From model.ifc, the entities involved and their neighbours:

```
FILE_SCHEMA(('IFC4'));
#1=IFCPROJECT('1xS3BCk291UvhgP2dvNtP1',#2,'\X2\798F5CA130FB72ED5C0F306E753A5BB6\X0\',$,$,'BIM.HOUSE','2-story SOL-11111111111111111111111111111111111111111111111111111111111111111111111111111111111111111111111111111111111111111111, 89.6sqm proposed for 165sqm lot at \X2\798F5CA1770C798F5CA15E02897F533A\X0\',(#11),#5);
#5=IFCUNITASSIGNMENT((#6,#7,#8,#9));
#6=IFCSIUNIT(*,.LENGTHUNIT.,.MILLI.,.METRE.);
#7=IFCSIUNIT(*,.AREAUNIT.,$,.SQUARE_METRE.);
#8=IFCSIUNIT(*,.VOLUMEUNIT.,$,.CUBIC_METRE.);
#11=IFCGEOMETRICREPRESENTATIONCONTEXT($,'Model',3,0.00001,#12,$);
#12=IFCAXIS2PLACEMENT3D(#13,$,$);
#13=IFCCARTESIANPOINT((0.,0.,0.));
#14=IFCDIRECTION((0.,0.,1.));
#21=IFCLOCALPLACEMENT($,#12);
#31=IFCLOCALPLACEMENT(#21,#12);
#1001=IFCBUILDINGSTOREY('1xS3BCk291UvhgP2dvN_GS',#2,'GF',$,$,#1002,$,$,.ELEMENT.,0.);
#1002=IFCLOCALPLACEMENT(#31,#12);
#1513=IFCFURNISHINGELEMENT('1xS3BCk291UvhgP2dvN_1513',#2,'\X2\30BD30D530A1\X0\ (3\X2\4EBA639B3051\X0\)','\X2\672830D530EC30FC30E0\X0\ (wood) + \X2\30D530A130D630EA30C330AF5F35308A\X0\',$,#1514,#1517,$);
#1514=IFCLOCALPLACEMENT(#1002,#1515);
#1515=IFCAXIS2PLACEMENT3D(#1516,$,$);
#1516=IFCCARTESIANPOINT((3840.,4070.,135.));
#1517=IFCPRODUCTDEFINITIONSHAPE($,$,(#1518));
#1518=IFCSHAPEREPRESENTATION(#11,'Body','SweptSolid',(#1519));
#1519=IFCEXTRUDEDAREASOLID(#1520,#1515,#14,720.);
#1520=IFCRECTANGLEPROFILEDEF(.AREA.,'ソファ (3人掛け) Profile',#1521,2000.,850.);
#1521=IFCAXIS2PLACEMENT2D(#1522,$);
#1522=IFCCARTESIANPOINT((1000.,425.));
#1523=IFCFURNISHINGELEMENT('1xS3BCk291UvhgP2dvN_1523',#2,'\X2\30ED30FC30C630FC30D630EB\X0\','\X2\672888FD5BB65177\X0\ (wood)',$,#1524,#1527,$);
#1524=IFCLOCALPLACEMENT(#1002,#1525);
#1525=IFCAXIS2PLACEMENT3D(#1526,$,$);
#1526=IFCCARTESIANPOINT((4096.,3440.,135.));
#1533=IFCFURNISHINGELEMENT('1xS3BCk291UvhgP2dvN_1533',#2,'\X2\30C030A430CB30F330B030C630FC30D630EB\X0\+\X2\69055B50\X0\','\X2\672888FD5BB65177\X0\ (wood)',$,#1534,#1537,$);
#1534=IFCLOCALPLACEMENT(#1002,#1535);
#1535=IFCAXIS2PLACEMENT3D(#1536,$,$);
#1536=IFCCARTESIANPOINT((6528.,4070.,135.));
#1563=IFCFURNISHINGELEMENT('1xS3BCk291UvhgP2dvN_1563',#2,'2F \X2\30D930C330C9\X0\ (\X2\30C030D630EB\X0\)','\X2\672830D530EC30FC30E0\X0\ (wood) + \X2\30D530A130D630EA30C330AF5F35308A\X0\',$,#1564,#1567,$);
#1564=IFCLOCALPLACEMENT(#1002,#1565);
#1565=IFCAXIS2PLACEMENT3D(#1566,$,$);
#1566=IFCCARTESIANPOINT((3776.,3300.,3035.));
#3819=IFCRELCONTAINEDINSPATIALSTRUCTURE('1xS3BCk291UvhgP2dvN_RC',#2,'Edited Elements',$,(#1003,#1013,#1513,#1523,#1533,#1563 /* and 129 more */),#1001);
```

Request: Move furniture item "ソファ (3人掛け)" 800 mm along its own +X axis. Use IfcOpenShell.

```python
import ifcopenshell
import ifcopenshell.api.geometry
import ifcopenshell.util.placement

model = ifcopenshell.open("model.ifc")

item = model.by_guid("1xS3BCk291UvhgP2dvN_1513")
matrix = ifcopenshell.util.placement.get_local_placement(item.ObjectPlacement)
matrix[:3, 3] += matrix[:3, 0] * 800.0
ifcopenshell.api.geometry.edit_object_placement(model, product=item, matrix=matrix, is_si=False)

print(ifcopenshell.util.placement.get_local_placement(item.ObjectPlacement).round(3) + 0.0)

model.write("model_rev.ifc")
```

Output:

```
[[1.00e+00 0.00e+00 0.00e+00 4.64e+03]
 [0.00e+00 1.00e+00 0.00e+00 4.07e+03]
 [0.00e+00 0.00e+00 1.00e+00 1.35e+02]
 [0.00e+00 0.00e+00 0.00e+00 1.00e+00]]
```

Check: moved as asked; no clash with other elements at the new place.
